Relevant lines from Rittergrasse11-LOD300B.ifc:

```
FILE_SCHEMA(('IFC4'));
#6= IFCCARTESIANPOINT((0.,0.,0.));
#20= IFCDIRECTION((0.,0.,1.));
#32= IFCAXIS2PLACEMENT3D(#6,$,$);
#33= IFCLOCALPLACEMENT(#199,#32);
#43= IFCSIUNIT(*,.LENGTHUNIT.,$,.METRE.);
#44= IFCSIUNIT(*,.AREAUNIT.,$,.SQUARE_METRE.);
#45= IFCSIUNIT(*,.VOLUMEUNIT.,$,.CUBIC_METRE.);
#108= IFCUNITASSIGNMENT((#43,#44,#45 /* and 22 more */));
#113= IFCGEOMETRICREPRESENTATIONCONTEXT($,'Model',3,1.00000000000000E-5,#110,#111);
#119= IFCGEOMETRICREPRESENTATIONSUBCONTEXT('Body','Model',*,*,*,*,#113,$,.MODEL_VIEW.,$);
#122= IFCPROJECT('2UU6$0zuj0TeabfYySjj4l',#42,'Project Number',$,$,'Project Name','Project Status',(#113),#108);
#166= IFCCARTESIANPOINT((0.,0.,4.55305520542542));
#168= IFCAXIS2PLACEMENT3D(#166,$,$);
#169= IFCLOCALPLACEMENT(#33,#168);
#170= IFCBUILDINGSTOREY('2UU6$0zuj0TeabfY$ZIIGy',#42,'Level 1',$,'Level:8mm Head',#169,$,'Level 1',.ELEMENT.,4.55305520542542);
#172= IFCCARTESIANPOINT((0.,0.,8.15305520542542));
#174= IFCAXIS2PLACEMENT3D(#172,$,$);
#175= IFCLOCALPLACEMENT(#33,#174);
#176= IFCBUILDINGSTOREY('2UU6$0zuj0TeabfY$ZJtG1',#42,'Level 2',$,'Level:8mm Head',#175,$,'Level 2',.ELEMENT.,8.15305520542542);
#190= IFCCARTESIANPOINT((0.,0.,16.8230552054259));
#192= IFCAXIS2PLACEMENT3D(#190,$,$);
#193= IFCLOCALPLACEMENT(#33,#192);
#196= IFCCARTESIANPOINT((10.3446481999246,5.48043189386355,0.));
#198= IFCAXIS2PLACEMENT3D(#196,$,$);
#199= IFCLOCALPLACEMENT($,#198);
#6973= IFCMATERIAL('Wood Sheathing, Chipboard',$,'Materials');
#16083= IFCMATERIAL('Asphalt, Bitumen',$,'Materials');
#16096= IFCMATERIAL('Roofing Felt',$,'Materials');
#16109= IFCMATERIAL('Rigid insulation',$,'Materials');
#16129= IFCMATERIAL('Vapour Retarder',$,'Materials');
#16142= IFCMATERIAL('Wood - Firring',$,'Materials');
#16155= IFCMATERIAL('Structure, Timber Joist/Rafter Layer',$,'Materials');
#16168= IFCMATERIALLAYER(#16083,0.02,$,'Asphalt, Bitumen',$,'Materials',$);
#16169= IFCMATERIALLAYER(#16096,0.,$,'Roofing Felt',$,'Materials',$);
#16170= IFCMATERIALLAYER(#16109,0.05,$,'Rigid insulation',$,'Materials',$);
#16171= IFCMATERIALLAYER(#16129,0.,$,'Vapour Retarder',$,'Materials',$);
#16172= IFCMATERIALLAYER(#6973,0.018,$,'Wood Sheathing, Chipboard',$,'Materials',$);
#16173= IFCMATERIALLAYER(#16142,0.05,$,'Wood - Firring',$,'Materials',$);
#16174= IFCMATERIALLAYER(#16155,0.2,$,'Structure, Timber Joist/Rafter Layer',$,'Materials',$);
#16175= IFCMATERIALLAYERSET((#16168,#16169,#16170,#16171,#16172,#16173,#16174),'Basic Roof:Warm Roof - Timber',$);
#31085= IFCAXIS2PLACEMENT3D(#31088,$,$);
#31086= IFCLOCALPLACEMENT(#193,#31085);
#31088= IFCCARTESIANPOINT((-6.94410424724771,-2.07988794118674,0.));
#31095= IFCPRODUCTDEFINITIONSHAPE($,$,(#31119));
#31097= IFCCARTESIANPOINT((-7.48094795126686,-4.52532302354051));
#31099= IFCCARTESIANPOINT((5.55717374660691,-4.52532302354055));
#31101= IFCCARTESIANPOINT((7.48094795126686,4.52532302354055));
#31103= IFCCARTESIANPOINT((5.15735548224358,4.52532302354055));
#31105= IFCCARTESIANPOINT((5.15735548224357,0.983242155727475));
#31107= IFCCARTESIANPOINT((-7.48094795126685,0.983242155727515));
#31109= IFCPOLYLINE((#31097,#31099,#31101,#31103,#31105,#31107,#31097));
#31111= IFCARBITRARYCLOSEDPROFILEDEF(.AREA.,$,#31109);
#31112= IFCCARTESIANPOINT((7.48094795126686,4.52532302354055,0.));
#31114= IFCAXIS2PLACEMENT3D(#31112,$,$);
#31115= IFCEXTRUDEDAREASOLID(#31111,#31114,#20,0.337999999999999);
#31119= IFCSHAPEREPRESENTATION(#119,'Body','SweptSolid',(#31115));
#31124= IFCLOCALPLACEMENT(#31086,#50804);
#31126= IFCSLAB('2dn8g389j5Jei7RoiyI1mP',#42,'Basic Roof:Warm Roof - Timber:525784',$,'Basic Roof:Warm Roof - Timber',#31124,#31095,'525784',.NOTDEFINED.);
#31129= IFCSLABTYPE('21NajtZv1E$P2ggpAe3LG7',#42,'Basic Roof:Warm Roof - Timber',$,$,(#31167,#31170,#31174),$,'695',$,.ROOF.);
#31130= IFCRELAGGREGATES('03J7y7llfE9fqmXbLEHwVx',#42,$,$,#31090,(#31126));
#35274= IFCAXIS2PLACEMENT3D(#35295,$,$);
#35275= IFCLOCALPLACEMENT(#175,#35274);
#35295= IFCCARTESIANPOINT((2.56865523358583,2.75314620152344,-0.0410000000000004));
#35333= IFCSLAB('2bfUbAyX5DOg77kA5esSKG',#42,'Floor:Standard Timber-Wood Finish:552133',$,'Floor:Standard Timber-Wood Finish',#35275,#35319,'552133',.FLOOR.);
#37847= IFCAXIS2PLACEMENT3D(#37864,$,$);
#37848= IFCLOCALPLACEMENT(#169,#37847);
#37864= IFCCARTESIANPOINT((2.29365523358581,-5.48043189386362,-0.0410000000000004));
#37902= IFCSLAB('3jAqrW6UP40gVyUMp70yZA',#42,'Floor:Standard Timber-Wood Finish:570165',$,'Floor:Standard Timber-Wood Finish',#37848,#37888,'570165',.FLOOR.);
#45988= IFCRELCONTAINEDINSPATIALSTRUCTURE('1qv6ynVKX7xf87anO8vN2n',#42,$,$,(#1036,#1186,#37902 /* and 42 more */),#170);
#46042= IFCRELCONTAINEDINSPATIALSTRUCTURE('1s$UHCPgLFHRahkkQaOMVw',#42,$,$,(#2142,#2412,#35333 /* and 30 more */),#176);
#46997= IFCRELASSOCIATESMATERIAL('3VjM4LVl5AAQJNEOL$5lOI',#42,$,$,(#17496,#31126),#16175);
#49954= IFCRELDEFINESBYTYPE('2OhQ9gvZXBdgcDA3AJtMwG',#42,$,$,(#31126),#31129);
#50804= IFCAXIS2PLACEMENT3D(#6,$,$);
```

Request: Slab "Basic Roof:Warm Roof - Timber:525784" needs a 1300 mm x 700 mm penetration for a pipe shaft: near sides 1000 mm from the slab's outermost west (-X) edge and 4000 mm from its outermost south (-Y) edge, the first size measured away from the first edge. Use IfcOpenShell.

```python
import numpy as np
import ifcopenshell
import ifcopenshell.api.feature
import ifcopenshell.api.geometry
import ifcopenshell.api.root
import ifcopenshell.geom
import ifcopenshell.util.placement
import ifcopenshell.util.representation
import ifcopenshell.util.shape
import ifcopenshell.util.unit

model = ifcopenshell.open("Rittergrasse11-LOD300B.ifc")
unit_scale = ifcopenshell.util.unit.calculate_unit_scale(model)
settings = ifcopenshell.geom.settings()


def volume(element):
    """Net volume in cubic metres, openings subtracted."""
    shape = ifcopenshell.geom.create_shape(settings, element)
    return ifcopenshell.util.shape.get_volume(shape.geometry)


slab = model.by_id(31126)
before = volume(slab)

# Extent in the slab's own axes, in metres. The edges named are its -X and -Y sides.
slab_shape = ifcopenshell.geom.create_shape(settings, slab)
vertices = ifcopenshell.util.shape.get_vertices(slab_shape.geometry)
x_min, y_min, bottom = vertices.min(axis=0)
top = vertices[:, 2].max()

opening = ifcopenshell.api.root.create_entity(model, ifc_class="IfcOpeningElement", name="Pipe shaft opening", predefined_type="OPENING")
context = ifcopenshell.util.representation.get_context(model, "Model", "Body", "MODEL_VIEW")
width, depth = 1.3, 0.7
outline = [(0.0, 0.0), (width, 0.0), (width, depth), (0.0, depth), (0.0, 0.0)]
# Overshoot both faces by 50 mm so the cut is clean.
shape = ifcopenshell.api.geometry.add_slab_representation(
    model, context=context, depth=top - bottom + 0.1, polyline=outline
)
ifcopenshell.api.geometry.assign_representation(model, product=opening, representation=shape)

matrix = ifcopenshell.util.placement.get_local_placement(slab.ObjectPlacement)
matrix[:, 3] = matrix @ np.append(np.array([x_min + 1, y_min + 4, bottom - 0.05]) / unit_scale, 1.0)
ifcopenshell.api.geometry.edit_object_placement(model, product=opening, matrix=matrix, is_si=False)
ifcopenshell.api.feature.add_feature(model, feature=opening, element=slab)

after = volume(slab)

print(f"slab volume {before:.3f} -> {after:.3f} m3")

model.write("Rittergrasse11-LOD300B-out.ifc")
```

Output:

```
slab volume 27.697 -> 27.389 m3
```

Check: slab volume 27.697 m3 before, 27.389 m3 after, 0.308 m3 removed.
